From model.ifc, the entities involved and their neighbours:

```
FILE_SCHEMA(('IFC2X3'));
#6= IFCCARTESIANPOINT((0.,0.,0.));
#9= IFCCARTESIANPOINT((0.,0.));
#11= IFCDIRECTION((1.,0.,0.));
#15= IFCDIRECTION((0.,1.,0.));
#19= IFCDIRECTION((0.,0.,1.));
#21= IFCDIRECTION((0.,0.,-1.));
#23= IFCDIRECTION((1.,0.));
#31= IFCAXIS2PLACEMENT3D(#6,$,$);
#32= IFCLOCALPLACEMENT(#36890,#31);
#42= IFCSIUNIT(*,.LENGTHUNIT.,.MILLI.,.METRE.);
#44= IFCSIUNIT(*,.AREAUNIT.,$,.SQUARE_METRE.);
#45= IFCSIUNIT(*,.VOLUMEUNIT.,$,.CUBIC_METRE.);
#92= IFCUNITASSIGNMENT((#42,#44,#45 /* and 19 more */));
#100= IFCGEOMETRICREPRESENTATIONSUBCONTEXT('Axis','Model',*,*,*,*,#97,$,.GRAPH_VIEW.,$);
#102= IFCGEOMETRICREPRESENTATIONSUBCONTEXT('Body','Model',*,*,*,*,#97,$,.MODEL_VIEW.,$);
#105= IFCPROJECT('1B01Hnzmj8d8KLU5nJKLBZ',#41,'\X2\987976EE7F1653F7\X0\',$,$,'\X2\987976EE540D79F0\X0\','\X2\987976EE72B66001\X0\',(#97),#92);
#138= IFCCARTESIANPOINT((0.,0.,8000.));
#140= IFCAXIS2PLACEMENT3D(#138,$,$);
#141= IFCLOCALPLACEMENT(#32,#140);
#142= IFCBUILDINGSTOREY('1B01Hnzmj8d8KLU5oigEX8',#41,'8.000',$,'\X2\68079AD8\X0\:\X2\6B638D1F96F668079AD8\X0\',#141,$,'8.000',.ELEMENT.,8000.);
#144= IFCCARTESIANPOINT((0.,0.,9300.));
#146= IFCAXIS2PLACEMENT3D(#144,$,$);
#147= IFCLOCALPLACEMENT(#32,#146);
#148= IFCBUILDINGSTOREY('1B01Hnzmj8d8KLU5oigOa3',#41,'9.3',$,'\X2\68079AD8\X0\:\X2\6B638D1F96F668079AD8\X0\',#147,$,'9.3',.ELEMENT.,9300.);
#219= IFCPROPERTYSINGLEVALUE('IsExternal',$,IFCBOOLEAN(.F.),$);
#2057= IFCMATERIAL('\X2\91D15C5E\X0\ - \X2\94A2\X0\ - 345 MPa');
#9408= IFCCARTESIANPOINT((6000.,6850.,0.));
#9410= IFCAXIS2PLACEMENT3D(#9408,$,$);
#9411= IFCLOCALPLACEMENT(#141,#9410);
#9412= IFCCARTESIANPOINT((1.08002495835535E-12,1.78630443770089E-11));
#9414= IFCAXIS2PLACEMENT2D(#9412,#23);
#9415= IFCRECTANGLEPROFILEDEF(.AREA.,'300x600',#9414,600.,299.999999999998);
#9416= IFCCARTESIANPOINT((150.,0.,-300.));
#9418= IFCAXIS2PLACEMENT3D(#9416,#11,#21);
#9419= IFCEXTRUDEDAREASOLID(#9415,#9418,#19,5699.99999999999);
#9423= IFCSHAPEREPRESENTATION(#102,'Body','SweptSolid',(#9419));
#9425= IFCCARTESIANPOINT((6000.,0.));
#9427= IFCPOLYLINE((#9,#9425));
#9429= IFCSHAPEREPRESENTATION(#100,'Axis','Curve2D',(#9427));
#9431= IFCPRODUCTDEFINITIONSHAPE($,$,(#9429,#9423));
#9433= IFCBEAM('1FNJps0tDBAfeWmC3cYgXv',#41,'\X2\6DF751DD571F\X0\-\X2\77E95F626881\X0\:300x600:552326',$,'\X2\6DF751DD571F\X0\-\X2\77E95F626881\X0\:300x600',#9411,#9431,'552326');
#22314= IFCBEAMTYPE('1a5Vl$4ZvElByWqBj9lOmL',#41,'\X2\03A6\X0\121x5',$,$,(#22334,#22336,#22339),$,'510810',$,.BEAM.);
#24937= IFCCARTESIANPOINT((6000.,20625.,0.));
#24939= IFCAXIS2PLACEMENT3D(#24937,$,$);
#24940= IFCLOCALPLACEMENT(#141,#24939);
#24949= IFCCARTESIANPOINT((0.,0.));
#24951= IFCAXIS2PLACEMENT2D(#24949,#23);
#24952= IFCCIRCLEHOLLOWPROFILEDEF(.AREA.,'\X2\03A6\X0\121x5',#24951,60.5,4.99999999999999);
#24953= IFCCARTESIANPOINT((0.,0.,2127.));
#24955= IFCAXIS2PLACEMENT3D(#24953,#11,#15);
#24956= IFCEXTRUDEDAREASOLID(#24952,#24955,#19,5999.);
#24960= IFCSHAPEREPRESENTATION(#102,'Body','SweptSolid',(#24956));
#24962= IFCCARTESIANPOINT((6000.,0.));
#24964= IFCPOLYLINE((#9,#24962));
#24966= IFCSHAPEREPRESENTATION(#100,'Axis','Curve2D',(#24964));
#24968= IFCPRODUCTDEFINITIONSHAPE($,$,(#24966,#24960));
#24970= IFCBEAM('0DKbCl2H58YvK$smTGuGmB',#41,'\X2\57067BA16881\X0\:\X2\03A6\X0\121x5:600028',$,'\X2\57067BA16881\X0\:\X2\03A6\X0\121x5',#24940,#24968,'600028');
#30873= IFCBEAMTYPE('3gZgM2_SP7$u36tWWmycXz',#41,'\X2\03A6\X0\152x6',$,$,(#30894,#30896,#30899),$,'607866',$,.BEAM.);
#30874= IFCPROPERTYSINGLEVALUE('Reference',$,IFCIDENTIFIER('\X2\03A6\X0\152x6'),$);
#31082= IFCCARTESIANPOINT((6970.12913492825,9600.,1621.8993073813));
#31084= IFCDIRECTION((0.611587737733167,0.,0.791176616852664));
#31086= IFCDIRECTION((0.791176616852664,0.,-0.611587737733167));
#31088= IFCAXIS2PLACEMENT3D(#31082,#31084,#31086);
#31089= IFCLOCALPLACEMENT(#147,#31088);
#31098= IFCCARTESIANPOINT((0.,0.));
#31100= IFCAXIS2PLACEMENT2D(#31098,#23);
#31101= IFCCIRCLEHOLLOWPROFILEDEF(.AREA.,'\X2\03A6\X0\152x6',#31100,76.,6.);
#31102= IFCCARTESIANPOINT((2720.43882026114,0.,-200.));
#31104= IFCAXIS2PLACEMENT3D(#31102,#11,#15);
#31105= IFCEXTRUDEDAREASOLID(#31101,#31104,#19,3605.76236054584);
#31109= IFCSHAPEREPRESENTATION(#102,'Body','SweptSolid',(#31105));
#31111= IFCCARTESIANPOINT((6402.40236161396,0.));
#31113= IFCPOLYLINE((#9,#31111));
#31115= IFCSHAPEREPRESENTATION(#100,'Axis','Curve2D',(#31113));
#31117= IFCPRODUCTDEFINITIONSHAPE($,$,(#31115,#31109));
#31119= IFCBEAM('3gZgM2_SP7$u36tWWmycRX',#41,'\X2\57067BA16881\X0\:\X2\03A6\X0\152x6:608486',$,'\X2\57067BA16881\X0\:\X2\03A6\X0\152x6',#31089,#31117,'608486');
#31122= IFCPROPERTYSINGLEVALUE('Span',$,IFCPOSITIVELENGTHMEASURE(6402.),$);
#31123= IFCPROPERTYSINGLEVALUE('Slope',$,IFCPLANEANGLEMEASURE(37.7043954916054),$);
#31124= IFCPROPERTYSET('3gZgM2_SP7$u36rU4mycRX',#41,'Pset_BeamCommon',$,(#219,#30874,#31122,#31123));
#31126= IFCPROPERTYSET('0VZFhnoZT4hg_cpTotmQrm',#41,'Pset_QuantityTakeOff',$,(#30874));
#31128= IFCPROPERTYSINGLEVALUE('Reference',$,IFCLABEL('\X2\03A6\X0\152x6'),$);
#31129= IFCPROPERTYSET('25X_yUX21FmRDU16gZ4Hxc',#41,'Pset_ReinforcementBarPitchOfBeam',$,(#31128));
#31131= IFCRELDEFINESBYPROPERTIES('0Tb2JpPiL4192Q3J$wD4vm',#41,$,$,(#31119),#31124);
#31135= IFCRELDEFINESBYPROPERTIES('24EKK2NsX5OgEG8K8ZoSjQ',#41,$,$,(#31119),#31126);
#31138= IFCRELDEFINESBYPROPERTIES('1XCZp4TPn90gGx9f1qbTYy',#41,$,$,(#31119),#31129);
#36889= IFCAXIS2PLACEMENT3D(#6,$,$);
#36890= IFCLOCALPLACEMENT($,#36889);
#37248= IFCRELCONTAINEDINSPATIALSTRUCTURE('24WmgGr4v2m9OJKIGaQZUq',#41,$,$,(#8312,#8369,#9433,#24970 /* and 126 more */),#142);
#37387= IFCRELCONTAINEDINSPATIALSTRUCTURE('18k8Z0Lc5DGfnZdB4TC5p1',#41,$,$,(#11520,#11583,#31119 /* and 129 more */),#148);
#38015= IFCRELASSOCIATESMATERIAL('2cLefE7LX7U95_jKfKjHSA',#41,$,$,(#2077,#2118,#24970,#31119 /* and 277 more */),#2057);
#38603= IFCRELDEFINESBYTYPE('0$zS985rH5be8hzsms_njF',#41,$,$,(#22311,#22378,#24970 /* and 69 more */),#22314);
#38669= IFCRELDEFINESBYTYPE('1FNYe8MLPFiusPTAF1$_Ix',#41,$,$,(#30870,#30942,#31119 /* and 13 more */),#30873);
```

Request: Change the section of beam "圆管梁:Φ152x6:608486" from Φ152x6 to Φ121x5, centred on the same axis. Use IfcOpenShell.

```python
import ifcopenshell
import ifcopenshell.api.pset
import ifcopenshell.api.type
import ifcopenshell.util.element
import ifcopenshell.util.representation

model = ifcopenshell.open("model.ifc")

member = model.by_id(31119)
source = next(p for p in model.by_type("IfcCircleHollowProfileDef") if p.ProfileName == "Φ121x5")

body = ifcopenshell.util.representation.get_representation(member, "Model", "Body")
solid = body.Items[0]
old_profile = solid.SweptArea

# Copy the section's sizes but keep this member's own profile position.
profile = ifcopenshell.util.element.copy(model, source)
profile.Position = old_profile.Position
solid.SweptArea = profile
if not model.get_total_inverses(old_profile):
    ifcopenshell.util.element.remove_deep2(model, old_profile)

new_type = model.by_guid("1a5Vl$4ZvElByWqBj9lOmL")
ifcopenshell.api.type.assign_type(
    model, related_objects=[member], relating_type=new_type, should_map_representations=False
)
member.Name = member.Name.replace("Φ152x6", "Φ121x5")
member.ObjectType = "圆管梁:Φ121x5"
pset = model.by_id(ifcopenshell.util.element.get_pset(member, "Pset_BeamCommon", should_inherit=False)["id"])
ifcopenshell.api.pset.edit_pset(model, pset=pset, properties={"Reference": "Φ121x5"})
pset = model.by_id(ifcopenshell.util.element.get_pset(member, "Pset_QuantityTakeOff", should_inherit=False)["id"])
ifcopenshell.api.pset.edit_pset(model, pset=pset, properties={"Reference": "Φ121x5"})
pset = model.by_id(ifcopenshell.util.element.get_pset(member, "Pset_ReinforcementBarPitchOfBeam", should_inherit=False)["id"])
ifcopenshell.api.pset.edit_pset(model, pset=pset, properties={"Reference": "Φ121x5"})

print(solid.SweptArea)

model.write("model_rev.ifc")
```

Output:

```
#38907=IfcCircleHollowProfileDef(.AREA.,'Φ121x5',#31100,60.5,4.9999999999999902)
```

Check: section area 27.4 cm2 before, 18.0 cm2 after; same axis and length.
